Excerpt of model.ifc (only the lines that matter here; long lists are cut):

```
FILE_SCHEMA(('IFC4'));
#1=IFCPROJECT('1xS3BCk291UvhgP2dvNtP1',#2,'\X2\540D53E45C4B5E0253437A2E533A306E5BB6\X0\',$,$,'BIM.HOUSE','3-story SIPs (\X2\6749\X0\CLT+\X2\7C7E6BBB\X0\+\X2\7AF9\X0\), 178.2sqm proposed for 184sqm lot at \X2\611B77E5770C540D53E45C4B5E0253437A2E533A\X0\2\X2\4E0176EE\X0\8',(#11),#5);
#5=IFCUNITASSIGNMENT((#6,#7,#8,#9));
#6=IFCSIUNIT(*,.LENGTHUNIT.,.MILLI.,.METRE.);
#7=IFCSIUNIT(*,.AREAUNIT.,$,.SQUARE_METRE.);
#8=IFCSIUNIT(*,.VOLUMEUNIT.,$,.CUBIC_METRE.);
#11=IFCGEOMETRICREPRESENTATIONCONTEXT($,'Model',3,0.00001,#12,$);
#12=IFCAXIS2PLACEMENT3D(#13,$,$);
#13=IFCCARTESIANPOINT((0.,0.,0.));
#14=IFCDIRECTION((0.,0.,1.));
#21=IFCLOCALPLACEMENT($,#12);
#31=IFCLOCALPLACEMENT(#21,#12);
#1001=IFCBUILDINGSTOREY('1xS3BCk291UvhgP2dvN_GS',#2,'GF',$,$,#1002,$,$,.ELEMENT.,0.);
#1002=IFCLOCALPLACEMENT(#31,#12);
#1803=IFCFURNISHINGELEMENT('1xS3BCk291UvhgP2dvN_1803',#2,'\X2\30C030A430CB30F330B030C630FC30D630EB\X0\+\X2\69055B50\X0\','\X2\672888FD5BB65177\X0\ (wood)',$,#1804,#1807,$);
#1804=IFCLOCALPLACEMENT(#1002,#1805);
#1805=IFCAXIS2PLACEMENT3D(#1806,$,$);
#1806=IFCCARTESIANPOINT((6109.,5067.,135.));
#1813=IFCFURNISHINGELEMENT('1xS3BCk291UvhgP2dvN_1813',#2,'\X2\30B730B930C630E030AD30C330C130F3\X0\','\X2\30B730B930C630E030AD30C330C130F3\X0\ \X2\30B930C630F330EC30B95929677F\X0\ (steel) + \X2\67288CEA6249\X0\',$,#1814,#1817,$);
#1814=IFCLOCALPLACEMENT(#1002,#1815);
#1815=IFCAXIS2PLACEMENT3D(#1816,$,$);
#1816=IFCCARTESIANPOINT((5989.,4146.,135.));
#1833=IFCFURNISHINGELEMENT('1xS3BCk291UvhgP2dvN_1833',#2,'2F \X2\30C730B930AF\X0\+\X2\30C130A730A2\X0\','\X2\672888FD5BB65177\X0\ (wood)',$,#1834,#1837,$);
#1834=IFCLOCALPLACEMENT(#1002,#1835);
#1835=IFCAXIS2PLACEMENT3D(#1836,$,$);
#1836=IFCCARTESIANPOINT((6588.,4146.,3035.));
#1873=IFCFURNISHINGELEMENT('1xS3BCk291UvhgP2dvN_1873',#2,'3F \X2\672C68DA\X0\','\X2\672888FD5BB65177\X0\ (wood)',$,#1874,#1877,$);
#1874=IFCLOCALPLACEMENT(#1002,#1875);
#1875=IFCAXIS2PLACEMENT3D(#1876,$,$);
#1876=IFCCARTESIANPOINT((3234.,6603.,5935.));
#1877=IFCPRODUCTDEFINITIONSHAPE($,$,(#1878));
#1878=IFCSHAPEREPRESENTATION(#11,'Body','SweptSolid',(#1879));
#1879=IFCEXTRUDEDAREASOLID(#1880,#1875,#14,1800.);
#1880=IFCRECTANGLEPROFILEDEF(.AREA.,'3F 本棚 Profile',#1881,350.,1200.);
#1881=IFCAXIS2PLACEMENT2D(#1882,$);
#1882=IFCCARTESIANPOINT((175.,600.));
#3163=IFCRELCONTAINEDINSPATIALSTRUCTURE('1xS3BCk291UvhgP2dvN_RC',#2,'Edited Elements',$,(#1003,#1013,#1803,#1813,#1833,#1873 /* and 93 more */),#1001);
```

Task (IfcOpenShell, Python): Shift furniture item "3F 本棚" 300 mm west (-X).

```python
import ifcopenshell
import ifcopenshell.api.geometry
import ifcopenshell.util.placement

model = ifcopenshell.open("model.ifc")

item = model.by_id(1873)
matrix = ifcopenshell.util.placement.get_local_placement(item.ObjectPlacement)
matrix[0, 3] -= 300.0
ifcopenshell.api.geometry.edit_object_placement(model, product=item, matrix=matrix, is_si=False)

print(ifcopenshell.util.placement.get_local_placement(item.ObjectPlacement).round(3) + 0.0)

model.write("model-out.ifc")
```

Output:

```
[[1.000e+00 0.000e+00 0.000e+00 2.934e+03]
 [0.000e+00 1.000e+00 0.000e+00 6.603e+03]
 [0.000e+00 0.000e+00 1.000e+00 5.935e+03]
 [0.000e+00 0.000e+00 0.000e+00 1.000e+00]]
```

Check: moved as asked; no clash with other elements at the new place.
